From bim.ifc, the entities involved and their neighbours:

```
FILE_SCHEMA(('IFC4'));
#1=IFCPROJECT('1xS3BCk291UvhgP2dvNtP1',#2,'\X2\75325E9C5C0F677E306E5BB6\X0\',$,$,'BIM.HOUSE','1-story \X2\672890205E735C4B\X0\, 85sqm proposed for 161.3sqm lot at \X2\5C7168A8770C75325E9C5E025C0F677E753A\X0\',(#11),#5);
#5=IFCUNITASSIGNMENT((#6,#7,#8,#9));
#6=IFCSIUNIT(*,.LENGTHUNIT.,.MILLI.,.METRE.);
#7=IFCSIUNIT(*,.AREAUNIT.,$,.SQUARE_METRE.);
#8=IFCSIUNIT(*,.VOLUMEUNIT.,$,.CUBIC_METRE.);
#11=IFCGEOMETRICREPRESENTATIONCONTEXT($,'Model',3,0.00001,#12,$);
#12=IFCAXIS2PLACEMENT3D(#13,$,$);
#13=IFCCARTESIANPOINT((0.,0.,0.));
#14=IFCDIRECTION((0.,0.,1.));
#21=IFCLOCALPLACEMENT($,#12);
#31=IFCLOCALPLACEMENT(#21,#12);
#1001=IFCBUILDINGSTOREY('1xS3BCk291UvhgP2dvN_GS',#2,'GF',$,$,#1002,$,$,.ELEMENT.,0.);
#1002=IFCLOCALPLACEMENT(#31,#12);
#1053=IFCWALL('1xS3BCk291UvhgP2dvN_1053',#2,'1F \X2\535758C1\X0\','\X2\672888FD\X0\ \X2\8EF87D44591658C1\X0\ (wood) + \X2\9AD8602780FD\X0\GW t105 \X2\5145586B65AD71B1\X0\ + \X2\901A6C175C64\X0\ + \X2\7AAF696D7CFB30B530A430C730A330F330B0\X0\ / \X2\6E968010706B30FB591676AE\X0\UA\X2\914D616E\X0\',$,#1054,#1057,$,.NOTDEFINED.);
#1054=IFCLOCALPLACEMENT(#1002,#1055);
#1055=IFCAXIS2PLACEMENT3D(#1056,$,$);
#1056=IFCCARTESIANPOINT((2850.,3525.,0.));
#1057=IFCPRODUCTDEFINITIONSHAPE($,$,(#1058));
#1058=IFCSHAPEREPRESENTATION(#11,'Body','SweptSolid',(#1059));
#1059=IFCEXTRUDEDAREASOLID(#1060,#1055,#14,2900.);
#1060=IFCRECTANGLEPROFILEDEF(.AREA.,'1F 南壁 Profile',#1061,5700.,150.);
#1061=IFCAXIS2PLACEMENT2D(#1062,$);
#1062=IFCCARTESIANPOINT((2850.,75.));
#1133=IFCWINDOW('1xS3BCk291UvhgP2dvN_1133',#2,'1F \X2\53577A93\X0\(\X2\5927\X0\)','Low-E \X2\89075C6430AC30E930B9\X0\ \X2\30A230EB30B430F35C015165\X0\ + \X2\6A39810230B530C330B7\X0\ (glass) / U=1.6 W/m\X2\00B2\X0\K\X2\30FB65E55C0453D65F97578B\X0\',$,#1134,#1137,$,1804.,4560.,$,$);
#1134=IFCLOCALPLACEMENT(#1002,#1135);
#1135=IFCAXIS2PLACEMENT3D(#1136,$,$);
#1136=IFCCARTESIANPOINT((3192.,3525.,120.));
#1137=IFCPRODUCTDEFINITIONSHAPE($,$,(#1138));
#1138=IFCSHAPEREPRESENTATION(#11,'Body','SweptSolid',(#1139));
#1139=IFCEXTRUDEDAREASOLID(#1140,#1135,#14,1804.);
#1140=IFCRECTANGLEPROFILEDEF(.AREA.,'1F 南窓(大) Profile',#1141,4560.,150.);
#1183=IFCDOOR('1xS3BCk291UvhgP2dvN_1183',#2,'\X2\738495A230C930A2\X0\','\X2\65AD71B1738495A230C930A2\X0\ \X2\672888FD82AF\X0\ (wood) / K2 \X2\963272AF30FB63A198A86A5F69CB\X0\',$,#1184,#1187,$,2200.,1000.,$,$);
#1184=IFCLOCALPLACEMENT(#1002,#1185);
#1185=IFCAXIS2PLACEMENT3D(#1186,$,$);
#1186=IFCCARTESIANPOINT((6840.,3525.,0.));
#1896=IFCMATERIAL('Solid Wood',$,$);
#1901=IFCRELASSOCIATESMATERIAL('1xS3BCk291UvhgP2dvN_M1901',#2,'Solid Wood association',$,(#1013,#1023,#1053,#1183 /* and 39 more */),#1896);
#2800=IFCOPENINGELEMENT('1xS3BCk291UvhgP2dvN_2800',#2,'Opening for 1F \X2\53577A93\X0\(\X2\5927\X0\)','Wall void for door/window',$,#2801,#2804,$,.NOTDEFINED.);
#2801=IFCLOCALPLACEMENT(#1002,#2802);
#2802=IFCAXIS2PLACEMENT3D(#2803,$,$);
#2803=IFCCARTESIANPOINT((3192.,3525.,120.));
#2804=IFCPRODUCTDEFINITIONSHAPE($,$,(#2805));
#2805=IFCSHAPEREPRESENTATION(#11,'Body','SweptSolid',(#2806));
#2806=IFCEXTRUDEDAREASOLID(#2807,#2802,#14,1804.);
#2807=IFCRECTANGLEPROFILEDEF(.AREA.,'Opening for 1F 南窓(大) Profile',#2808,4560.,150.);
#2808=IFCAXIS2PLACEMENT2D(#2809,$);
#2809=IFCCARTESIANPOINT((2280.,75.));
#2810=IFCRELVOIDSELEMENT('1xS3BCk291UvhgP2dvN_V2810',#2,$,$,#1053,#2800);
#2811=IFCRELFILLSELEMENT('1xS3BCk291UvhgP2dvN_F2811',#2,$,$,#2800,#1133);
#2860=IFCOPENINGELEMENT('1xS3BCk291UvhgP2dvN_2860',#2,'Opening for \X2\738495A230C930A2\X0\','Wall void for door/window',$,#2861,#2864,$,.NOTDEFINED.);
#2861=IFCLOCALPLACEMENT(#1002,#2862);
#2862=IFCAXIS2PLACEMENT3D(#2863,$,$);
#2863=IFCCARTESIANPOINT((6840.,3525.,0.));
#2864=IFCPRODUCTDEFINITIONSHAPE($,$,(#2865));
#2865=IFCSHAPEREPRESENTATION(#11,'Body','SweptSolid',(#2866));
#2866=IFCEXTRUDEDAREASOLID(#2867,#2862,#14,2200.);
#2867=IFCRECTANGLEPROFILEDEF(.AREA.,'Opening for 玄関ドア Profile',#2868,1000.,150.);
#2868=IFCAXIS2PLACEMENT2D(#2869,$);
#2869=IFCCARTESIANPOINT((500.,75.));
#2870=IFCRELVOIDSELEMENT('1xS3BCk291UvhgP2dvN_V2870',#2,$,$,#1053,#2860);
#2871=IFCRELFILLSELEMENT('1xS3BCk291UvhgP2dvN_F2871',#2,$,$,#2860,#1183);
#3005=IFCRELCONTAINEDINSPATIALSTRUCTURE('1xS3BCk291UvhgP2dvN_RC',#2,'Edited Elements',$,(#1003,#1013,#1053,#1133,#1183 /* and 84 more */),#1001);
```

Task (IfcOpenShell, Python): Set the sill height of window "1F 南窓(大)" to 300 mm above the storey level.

```python
import numpy as np
import ifcopenshell
import ifcopenshell.api.geometry
import ifcopenshell.geom
import ifcopenshell.util.element
import ifcopenshell.util.placement
import ifcopenshell.util.shape
import ifcopenshell.util.unit

model = ifcopenshell.open("bim.ifc")
unit_scale = ifcopenshell.util.unit.calculate_unit_scale(model)

window = model.by_guid("1xS3BCk291UvhgP2dvN_1133")
opening = window.FillsVoids[0].RelatingOpeningElement
storey = ifcopenshell.util.element.get_container(window, ifc_class="IfcBuildingStorey")
level = ifcopenshell.util.placement.get_local_placement(storey.ObjectPlacement)[2, 3]

# The opening's origin need not be at the sill, so measure its lowest point.
shape = ifcopenshell.geom.create_shape(ifcopenshell.geom.settings(), opening)
bottom = ifcopenshell.util.shape.get_shape_bottom_elevation(shape, shape.geometry) / unit_scale
dz = level + 0.3 / unit_scale - bottom

shift = np.array([0.0, 0.0, dz])
# The window is not placed relative to its opening, so move both.
for product in (opening, window):
    matrix = ifcopenshell.util.placement.get_local_placement(product.ObjectPlacement)
    matrix[:3, 3] += shift
    ifcopenshell.api.geometry.edit_object_placement(model, product=product, matrix=matrix, is_si=False)

print(f"moved by {dz * unit_scale:+.3f} m")

model.write("bim_v2.ifc")
```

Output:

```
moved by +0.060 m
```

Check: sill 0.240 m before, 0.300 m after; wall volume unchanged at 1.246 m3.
